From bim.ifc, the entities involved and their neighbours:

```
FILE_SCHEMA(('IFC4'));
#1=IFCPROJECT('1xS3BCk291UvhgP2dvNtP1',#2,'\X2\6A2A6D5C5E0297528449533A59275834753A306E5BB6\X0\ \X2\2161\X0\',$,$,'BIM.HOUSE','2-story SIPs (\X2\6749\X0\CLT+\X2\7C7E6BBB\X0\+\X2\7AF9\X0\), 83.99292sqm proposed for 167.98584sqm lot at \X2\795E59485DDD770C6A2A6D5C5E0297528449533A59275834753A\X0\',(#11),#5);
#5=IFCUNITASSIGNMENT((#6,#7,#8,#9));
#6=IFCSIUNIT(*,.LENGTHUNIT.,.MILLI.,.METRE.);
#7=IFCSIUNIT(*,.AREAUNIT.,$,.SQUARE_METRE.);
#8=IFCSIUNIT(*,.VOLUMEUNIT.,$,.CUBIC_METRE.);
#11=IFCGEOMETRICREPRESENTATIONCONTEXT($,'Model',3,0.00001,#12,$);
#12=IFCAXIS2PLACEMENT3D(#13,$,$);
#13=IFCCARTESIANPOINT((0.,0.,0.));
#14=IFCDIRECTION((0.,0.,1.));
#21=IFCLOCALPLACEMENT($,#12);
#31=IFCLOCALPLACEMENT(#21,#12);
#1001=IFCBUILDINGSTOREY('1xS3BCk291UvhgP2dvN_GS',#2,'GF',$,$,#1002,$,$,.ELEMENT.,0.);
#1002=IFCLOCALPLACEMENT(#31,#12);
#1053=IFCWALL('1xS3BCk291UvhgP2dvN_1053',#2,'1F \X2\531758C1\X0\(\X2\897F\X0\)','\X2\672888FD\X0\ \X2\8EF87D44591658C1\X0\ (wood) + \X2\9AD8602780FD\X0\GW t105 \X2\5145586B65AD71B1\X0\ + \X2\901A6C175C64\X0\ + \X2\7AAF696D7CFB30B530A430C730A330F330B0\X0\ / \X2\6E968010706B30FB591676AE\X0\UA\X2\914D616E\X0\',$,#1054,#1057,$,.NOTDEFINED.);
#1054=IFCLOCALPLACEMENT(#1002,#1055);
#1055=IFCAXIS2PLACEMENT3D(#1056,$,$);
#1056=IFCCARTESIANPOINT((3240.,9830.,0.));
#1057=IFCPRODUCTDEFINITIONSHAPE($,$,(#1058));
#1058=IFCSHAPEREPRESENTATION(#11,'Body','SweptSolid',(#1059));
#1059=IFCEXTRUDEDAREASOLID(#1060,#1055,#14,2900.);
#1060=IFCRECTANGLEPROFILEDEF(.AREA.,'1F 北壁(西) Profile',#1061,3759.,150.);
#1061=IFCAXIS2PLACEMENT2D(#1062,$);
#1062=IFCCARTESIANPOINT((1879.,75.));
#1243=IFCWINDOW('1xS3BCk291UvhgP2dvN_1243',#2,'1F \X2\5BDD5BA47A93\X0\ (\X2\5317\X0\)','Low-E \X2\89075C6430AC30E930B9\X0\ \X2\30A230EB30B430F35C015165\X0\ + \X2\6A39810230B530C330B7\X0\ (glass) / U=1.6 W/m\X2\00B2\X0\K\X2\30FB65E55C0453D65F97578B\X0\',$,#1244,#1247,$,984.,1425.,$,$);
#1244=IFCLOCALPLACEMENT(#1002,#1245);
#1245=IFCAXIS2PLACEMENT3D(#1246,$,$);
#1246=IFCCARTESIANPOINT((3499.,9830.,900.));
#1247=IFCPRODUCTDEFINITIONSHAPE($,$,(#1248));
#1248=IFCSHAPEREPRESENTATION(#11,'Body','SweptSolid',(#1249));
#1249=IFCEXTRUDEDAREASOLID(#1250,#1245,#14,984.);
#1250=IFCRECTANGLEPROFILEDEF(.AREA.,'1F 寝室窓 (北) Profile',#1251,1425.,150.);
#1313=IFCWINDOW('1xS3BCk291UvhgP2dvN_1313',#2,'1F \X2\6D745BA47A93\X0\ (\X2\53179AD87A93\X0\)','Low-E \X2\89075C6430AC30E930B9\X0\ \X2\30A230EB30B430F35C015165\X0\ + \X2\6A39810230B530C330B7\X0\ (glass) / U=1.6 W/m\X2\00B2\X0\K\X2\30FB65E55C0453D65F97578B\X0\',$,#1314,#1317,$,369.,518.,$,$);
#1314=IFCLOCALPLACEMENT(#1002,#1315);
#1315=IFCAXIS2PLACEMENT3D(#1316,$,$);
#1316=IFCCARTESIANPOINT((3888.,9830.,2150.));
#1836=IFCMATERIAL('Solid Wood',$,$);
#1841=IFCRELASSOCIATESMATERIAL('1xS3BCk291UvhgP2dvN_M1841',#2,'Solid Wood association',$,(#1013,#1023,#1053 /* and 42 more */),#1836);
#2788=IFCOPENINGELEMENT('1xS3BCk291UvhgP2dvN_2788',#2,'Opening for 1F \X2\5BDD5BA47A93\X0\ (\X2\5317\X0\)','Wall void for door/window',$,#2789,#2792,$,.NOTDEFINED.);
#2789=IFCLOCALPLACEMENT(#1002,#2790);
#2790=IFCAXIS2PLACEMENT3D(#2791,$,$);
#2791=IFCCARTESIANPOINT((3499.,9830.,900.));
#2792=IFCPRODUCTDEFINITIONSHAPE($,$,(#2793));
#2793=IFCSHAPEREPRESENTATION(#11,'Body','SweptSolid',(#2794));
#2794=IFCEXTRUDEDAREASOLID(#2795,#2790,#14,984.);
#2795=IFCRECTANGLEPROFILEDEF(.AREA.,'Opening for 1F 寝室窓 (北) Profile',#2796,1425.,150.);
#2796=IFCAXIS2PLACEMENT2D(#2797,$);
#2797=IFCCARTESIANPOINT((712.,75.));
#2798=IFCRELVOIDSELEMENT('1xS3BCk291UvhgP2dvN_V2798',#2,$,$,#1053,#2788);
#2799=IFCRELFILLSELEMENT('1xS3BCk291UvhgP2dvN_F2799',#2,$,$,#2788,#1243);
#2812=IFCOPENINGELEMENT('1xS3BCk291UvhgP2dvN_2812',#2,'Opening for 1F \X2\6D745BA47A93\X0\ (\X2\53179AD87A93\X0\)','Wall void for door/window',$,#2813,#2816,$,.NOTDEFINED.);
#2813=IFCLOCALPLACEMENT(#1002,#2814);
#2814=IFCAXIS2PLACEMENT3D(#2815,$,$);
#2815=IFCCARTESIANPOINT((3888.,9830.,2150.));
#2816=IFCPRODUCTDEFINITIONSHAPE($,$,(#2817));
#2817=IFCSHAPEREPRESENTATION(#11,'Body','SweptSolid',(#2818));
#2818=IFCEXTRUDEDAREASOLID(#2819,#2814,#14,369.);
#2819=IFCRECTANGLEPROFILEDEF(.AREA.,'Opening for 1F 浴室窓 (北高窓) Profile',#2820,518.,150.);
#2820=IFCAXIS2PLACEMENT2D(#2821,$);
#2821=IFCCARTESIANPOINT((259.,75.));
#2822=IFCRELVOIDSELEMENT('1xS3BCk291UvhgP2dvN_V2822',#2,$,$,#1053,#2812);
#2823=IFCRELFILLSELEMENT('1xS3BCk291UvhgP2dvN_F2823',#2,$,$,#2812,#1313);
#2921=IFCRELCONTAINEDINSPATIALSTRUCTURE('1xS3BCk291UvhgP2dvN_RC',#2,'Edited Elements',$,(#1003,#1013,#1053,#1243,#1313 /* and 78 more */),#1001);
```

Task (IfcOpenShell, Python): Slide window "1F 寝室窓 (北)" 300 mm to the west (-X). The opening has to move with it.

```python
import ifcopenshell
import ifcopenshell.api.geometry
import ifcopenshell.util.placement
import ifcopenshell.util.unit

model = ifcopenshell.open("bim.ifc")
unit_scale = ifcopenshell.util.unit.calculate_unit_scale(model)

window = model.by_guid("1xS3BCk291UvhgP2dvN_1243")
opening = window.FillsVoids[0].RelatingOpeningElement
wall = opening.VoidsElements[0].RelatingBuildingElement

wall_matrix = ifcopenshell.util.placement.get_local_placement(wall.ObjectPlacement)
shift = wall_matrix[:3, 0] * -0.3 / unit_scale
before = ifcopenshell.util.placement.get_local_placement(window.ObjectPlacement)[:3, 3].copy()

# The window is not placed relative to its opening, so move both.
for product in (opening, window):
    matrix = ifcopenshell.util.placement.get_local_placement(product.ObjectPlacement)
    matrix[:3, 3] += shift
    ifcopenshell.api.geometry.edit_object_placement(model, product=product, matrix=matrix, is_si=False)

after = ifcopenshell.util.placement.get_local_placement(window.ObjectPlacement)[:3, 3]
print("window moved by", (after - before).round(3) + 0.0)

model.write("bim_updated.ifc")
```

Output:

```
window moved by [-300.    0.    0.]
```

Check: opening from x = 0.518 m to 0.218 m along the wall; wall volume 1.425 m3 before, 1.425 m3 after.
